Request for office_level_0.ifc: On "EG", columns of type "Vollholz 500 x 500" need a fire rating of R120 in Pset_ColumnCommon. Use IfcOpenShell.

First a look at what the model holds.

```python
import ifcopenshell
import ifcopenshell.util.element

model = ifcopenshell.open("office_level_0.ifc")
print(model.schema)
storey = next(s for s in model.by_type("IfcBuildingStorey") if s.Name == "EG")
columns = [e for e in ifcopenshell.util.element.get_decomposition(storey) if e.is_a("IfcColumn")]
seen = {}
for e in columns:
    element_type = ifcopenshell.util.element.get_type(e)
    key = (element_type.Name if element_type != e and element_type else None, ifcopenshell.util.element.get_pset(e, "Pset_ColumnCommon", "FireRating"))
    seen[key] = seen.get(key, 0) + 1
for (name, value), count in sorted(seen.items(), key=str):
    print(count, "x", name, "|", value)
```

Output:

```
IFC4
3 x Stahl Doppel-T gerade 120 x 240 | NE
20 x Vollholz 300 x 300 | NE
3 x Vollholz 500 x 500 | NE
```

```python
import ifcopenshell
import ifcopenshell.api.pset
import ifcopenshell.util.element

model = ifcopenshell.open("office_level_0.ifc")

storey = next(s for s in model.by_type("IfcBuildingStorey") if s.Name == "EG")
columns = [e for e in ifcopenshell.util.element.get_decomposition(storey) if e.is_a("IfcColumn")]

count = 0
for e in columns:
    element_type = ifcopenshell.util.element.get_type(e)
    if element_type in (None, e) or element_type.Name != "Vollholz 500 x 500":
        continue
    # add_pset returns the element's existing set when there is one.
    pset = ifcopenshell.api.pset.add_pset(model, product=e, name="Pset_ColumnCommon")
    ifcopenshell.api.pset.edit_pset(model, pset=pset, properties={"FireRating": "R120"})
    count += 1

print(count, "columns updated")

model.write("office_level_0_edited.ifc")
```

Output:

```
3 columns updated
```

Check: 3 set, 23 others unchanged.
